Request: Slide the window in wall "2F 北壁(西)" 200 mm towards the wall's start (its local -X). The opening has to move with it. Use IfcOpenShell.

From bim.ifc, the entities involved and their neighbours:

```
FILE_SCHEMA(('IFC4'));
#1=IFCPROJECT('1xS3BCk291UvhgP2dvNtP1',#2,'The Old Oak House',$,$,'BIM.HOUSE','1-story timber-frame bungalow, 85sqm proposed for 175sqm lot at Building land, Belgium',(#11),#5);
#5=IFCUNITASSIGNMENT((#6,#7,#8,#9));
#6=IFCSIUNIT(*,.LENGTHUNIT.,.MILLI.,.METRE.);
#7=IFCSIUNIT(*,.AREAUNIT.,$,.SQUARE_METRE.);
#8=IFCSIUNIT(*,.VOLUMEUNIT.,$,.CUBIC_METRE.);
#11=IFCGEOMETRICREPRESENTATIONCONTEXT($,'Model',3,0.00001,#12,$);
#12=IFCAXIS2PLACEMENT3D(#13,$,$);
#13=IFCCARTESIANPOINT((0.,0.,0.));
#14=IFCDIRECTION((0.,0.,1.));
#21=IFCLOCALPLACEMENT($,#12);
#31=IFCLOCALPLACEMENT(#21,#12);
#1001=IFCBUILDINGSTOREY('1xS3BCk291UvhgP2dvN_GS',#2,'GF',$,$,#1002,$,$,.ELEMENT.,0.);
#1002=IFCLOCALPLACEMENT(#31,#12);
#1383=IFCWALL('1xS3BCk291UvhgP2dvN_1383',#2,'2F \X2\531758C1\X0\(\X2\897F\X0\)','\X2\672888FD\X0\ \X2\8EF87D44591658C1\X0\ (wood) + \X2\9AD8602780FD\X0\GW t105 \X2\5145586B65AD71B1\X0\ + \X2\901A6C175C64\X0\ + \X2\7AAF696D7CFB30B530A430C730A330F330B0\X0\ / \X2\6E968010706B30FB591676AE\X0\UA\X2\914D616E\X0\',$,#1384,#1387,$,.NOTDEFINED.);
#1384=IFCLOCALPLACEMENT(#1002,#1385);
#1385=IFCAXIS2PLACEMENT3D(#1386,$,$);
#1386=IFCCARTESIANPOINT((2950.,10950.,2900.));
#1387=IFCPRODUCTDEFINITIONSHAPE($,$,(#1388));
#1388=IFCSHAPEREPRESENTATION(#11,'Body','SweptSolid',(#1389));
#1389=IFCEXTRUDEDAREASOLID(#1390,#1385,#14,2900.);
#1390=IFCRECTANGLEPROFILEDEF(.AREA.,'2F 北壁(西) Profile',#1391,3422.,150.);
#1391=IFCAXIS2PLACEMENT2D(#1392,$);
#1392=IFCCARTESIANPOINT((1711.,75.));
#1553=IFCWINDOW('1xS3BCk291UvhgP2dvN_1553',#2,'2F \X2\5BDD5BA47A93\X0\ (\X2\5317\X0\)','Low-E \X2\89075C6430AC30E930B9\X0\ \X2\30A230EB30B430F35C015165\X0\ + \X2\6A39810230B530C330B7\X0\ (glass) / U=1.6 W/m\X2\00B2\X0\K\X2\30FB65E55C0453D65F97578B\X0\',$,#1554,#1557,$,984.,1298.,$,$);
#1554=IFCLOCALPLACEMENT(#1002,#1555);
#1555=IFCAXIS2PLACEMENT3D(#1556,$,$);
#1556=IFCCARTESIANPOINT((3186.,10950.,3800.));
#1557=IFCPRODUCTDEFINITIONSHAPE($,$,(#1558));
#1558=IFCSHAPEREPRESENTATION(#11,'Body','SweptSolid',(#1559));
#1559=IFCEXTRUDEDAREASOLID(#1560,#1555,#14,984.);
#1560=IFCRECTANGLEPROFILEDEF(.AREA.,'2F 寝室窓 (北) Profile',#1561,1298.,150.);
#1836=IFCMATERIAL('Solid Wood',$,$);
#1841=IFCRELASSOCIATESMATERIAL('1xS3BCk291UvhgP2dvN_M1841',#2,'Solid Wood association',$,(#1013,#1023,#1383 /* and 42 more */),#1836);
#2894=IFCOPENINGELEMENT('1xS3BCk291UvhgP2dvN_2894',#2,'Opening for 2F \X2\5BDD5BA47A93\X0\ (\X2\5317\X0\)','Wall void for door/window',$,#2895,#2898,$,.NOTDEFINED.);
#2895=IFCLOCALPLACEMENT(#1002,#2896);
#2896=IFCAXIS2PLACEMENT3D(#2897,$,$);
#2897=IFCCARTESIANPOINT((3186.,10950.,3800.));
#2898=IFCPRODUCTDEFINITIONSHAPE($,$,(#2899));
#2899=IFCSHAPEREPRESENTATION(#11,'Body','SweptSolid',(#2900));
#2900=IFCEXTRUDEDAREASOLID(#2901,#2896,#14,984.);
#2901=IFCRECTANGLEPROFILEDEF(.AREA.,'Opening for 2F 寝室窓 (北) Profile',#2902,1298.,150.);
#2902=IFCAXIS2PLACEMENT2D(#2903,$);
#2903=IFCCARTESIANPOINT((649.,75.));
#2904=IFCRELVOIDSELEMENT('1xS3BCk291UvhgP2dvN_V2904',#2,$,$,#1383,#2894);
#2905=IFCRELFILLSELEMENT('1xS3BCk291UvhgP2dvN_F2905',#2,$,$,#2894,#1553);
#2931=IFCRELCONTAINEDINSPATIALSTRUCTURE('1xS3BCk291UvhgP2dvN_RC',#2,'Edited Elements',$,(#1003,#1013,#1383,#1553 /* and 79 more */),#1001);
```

```python
import ifcopenshell
import ifcopenshell.api.geometry
import ifcopenshell.util.placement
import ifcopenshell.util.unit

model = ifcopenshell.open("bim.ifc")
unit_scale = ifcopenshell.util.unit.calculate_unit_scale(model)

window = model.by_guid("1xS3BCk291UvhgP2dvN_1553")
opening = window.FillsVoids[0].RelatingOpeningElement
wall = opening.VoidsElements[0].RelatingBuildingElement

wall_matrix = ifcopenshell.util.placement.get_local_placement(wall.ObjectPlacement)
shift = wall_matrix[:3, 0] * -0.2 / unit_scale
before = ifcopenshell.util.placement.get_local_placement(window.ObjectPlacement)[:3, 3].copy()

# The window is not placed relative to its opening, so move both.
for product in (opening, window):
    matrix = ifcopenshell.util.placement.get_local_placement(product.ObjectPlacement)
    matrix[:3, 3] += shift
    ifcopenshell.api.geometry.edit_object_placement(model, product=product, matrix=matrix, is_si=False)

after = ifcopenshell.util.placement.get_local_placement(window.ObjectPlacement)[:3, 3]
print("window moved by", (after - before).round(3) + 0.0)

model.write("bim_rev.ifc")
```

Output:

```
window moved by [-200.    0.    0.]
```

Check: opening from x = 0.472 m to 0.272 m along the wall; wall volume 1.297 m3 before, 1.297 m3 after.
